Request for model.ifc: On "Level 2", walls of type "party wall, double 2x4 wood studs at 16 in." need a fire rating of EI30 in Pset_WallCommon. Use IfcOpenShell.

First a look at what the model holds.

```python
import ifcopenshell
import ifcopenshell.util.element

model = ifcopenshell.open("model.ifc")
print(model.schema)
storey = next(s for s in model.by_type("IfcBuildingStorey") if s.Name == "Level 2")
walls = [e for e in ifcopenshell.util.element.get_decomposition(storey) if e.is_a("IfcWall")]
seen = {}
for e in walls:
    element_type = ifcopenshell.util.element.get_type(e)
    key = (element_type.Name if element_type != e and element_type else None, ifcopenshell.util.element.get_pset(e, "Pset_WallCommon", "FireRating"))
    seen[key] = seen.get(key, 0) + 1
for (name, value), count in sorted(seen.items(), key=str):
    print(count, "x", name, "|", value)
```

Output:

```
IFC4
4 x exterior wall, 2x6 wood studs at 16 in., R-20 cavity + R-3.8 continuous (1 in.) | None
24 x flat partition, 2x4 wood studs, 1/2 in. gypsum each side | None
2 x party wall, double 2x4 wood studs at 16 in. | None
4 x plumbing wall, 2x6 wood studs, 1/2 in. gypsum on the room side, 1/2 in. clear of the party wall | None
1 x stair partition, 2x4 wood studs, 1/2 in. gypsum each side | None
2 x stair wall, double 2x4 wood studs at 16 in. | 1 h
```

```python
import ifcopenshell
import ifcopenshell.api.pset
import ifcopenshell.util.element

model = ifcopenshell.open("model.ifc")

storey = next(s for s in model.by_type("IfcBuildingStorey") if s.Name == "Level 2")
walls = [e for e in ifcopenshell.util.element.get_decomposition(storey) if e.is_a("IfcWall")]

count = 0
for e in walls:
    element_type = ifcopenshell.util.element.get_type(e)
    if element_type in (None, e) or element_type.Name != "party wall, double 2x4 wood studs at 16 in.":
        continue
    # add_pset returns the element's existing set when there is one.
    pset = ifcopenshell.api.pset.add_pset(model, product=e, name="Pset_WallCommon")
    ifcopenshell.api.pset.edit_pset(model, pset=pset, properties={"FireRating": "EI30"})
    count += 1

print(count, "walls updated")

model.write("model_rev.ifc")
```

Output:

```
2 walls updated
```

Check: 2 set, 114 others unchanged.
